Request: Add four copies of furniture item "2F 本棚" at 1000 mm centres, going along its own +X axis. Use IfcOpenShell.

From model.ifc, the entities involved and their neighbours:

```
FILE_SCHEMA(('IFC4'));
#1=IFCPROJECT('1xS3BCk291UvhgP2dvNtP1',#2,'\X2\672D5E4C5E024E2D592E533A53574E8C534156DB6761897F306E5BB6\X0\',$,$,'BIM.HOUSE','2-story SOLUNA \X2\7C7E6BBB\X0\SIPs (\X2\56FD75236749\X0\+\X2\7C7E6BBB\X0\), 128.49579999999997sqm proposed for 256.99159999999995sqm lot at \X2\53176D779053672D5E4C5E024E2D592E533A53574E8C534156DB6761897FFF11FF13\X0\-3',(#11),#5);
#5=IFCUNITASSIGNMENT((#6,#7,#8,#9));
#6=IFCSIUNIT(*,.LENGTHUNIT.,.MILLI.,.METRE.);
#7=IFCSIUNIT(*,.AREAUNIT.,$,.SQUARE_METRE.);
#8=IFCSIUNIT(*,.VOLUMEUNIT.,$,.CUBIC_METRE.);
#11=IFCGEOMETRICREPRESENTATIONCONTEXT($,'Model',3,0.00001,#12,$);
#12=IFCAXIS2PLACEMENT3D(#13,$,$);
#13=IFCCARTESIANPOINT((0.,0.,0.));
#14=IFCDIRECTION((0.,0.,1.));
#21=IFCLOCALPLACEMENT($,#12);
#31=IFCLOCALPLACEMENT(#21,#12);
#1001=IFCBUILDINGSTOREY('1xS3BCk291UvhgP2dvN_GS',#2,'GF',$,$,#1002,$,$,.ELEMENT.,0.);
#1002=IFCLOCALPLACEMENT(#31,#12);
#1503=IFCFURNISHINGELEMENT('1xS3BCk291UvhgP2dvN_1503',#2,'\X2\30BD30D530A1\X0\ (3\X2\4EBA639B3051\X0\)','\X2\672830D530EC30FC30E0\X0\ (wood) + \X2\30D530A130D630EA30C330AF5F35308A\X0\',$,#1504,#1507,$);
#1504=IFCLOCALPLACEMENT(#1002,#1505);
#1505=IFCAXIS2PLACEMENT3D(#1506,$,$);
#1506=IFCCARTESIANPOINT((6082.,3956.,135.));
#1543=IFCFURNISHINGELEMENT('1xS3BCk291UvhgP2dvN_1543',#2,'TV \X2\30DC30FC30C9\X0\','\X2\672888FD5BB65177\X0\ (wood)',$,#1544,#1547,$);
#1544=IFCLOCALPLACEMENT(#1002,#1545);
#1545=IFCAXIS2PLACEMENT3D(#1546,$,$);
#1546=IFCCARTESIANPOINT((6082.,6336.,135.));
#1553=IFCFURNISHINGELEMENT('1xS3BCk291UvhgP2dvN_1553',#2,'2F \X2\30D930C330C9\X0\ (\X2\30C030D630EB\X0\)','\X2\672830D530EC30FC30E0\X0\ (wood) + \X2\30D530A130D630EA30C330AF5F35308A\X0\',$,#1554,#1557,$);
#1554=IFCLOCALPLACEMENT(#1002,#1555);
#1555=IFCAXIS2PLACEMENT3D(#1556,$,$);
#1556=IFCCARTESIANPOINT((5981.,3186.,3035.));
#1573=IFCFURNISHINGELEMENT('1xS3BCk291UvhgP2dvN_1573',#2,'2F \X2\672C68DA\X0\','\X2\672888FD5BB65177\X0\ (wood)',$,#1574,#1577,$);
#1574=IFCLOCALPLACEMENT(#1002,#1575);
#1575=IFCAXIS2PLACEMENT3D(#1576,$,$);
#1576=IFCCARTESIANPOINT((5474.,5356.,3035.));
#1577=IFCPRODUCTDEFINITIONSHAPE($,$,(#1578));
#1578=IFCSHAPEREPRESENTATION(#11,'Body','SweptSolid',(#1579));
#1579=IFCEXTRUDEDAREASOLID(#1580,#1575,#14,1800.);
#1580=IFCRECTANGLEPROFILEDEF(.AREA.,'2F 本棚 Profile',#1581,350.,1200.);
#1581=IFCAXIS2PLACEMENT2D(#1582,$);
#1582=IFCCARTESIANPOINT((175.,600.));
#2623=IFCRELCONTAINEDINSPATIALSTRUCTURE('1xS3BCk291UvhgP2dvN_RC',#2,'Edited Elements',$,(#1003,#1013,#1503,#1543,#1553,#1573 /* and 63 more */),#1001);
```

```python
import ifcopenshell
import ifcopenshell.api.geometry
import ifcopenshell.api.root
import ifcopenshell.util.element
import ifcopenshell.util.placement

model = ifcopenshell.open("model.ifc")


def reuse_history(source, copy):
    """copy_class also copies each property set's owner history, people and application; keep the originals."""
    for rel in copy.IsDefinedBy:
        if rel.is_a("IfcRelDefinesByProperties") and (history := rel.RelatingPropertyDefinition.OwnerHistory):
            rel.RelatingPropertyDefinition.OwnerHistory = source.OwnerHistory
            ifcopenshell.util.element.remove_deep2(model, history)


source = model.by_guid("1xS3BCk291UvhgP2dvN_1573")
base = ifcopenshell.util.placement.get_local_placement(source.ObjectPlacement)
step = base[:3, 0] * 1000.0

for i in range(1, 5):
    copy = ifcopenshell.api.root.copy_class(model, product=source)
    copy.Representation = ifcopenshell.util.element.copy_deep(
        model, source.Representation, exclude=["IfcGeometricRepresentationContext", "IfcRepresentationMap"]
    )
    reuse_history(source, copy)
    matrix = base.copy()
    matrix[:3, 3] += i * step
    print("added at", matrix[:3, 3].round(3) + 0.0)
    ifcopenshell.api.geometry.edit_object_placement(model, product=copy, matrix=matrix, is_si=False)

model.write("model_rev.ifc")
```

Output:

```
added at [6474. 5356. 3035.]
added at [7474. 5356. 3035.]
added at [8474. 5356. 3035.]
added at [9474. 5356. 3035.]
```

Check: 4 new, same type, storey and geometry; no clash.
